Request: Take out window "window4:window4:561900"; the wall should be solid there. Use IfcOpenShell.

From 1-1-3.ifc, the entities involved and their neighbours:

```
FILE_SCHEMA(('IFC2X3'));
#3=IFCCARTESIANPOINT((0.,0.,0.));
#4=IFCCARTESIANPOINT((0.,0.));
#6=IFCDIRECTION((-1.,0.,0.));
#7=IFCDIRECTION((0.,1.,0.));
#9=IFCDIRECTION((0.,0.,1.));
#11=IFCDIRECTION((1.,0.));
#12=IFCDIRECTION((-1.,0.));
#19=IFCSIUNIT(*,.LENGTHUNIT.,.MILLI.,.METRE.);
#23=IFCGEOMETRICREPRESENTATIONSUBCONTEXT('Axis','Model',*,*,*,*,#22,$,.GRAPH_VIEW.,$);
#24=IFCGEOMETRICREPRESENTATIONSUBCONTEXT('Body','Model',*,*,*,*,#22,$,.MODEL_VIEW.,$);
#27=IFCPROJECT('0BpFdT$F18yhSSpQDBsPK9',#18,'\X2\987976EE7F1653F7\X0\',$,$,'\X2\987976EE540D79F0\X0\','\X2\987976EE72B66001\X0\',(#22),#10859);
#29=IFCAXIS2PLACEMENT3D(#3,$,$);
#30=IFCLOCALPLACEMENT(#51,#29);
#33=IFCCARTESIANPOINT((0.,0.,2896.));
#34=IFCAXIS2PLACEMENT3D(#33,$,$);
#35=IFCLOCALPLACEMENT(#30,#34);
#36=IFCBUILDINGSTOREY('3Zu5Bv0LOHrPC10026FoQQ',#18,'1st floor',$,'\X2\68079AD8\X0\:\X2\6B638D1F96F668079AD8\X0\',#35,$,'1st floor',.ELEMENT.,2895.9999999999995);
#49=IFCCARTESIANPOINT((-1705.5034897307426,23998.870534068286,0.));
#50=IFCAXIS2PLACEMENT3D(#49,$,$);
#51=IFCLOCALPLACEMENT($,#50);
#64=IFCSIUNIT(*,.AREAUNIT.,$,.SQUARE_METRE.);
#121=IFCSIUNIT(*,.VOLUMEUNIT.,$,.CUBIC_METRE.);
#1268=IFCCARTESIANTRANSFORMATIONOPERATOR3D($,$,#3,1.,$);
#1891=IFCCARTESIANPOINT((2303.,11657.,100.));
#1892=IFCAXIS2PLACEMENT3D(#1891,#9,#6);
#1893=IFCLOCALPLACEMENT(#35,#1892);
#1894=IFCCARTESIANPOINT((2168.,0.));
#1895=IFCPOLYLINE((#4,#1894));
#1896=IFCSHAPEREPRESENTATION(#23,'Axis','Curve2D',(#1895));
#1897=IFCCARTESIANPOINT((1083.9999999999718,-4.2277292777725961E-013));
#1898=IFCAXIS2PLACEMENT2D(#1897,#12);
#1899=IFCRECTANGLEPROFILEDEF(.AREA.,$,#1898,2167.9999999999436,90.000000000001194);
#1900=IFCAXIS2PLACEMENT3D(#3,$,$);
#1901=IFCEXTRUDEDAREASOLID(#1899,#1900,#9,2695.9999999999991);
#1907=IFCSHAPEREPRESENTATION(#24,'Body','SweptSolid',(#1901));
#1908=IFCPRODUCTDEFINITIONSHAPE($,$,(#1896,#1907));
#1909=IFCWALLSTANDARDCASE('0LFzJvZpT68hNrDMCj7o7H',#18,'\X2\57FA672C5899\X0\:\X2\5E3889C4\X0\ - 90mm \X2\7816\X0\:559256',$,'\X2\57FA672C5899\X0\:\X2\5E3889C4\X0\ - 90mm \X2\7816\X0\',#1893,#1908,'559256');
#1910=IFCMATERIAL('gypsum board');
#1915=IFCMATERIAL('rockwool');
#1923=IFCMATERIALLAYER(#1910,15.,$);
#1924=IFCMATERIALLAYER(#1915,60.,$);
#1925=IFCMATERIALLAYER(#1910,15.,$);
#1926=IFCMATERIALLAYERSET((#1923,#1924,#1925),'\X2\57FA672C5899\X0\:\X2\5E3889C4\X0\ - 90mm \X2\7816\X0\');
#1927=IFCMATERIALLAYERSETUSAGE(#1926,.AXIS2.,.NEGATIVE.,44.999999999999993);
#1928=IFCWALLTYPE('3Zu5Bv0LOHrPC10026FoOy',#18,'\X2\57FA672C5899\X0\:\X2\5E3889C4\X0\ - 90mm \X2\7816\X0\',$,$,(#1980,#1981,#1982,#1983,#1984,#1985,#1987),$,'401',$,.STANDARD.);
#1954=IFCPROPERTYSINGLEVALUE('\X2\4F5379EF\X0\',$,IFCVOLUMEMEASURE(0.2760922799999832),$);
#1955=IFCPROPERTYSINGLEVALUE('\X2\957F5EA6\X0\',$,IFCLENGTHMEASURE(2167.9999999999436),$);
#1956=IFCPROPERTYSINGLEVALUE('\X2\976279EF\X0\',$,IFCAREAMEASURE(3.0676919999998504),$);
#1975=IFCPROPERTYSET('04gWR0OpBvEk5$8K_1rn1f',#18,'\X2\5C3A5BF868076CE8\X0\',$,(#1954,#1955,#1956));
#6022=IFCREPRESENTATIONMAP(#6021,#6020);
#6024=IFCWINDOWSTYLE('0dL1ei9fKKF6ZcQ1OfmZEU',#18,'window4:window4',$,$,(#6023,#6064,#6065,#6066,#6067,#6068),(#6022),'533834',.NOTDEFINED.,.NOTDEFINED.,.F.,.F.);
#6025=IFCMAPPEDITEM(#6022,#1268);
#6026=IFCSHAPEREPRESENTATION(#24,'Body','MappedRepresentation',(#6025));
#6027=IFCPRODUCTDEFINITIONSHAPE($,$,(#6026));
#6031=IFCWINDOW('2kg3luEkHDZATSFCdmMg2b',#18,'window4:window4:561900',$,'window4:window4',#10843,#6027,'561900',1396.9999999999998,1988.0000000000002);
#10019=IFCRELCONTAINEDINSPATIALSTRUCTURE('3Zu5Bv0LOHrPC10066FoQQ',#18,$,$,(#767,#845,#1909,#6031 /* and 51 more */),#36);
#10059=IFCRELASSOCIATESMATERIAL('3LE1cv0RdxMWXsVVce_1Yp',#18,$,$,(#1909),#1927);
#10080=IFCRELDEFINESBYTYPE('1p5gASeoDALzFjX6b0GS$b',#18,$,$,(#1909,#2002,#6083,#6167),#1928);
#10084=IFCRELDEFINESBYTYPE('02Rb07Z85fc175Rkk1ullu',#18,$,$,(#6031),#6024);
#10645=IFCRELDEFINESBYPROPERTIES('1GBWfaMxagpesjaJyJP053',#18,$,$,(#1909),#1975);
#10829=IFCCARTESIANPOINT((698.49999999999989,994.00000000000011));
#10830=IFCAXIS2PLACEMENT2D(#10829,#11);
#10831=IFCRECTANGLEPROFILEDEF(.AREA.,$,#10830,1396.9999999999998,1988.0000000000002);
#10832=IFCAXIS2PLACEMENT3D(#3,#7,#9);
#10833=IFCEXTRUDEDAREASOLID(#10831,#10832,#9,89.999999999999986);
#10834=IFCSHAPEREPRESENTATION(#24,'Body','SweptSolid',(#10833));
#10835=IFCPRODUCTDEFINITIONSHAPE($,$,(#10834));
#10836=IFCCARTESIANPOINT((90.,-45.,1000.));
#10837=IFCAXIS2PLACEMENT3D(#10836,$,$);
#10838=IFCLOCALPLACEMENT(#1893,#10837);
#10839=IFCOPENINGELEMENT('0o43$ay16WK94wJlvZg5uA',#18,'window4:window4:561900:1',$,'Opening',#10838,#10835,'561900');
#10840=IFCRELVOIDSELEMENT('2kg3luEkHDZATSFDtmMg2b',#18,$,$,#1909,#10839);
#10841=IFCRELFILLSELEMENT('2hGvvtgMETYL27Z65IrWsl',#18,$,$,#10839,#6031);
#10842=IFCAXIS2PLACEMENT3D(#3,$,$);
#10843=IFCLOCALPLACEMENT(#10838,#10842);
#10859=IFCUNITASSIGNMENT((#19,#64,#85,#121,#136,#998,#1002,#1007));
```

```python
import ifcopenshell
import ifcopenshell.api.feature
import ifcopenshell.api.pset
import ifcopenshell.api.root
import ifcopenshell.geom
import ifcopenshell.util.element
import ifcopenshell.util.shape
import ifcopenshell.util.unit

model = ifcopenshell.open("1-1-3.ifc")
area_scale = ifcopenshell.util.unit.calculate_unit_scale(model, "AREAUNIT")
volume_scale = ifcopenshell.util.unit.calculate_unit_scale(model, "VOLUMEUNIT")
settings = ifcopenshell.geom.settings()


def volume(element):
    """Net volume in cubic metres, openings subtracted."""
    shape = ifcopenshell.geom.create_shape(settings, element)
    return ifcopenshell.util.shape.get_volume(shape.geometry)


window = model.by_id(6031)
opening = window.FillsVoids[0].RelatingOpeningElement
wall = opening.VoidsElements[0].RelatingBuildingElement
before = volume(wall)

ifcopenshell.api.root.remove_product(model, product=window)
ifcopenshell.api.feature.remove_feature(model, feature=opening)

after = volume(wall)
thickness = 0.09  # wall thickness in metres

# Update the wall's stored quantities.
pset = model.by_id(ifcopenshell.util.element.get_pset(wall, "尺寸标注", should_inherit=False)["id"])
ifcopenshell.api.pset.edit_pset(model, pset=pset, properties={
    "体积": model.create_entity("IfcVolumeMeasure", after / volume_scale),
    "面积": model.create_entity("IfcAreaMeasure", after / thickness / area_scale),
})

print(f"wall volume {before:.3f} -> {after:.3f} m3")

model.write("1-1-3-out.ifc")
```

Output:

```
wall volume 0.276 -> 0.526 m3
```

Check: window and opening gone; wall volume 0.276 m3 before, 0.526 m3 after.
